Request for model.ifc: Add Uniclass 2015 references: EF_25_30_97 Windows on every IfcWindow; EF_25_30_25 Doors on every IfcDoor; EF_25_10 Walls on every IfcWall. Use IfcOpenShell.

First a look at what the model holds.

```python
import ifcopenshell

model = ifcopenshell.open("model.ifc")
print(model.schema)
print("classifications:", [c.Name for c in model.by_type("IfcClassification")])
for ifc_class in ("IfcDoor", "IfcRoof", "IfcStair", "IfcWall", "IfcWindow"):
    print(ifc_class, len(model.by_type(ifc_class)))
```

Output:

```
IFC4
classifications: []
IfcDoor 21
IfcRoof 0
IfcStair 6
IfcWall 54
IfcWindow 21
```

```python
import ifcopenshell
import ifcopenshell.api.classification

model = ifcopenshell.open("model.ifc")

system = ifcopenshell.api.classification.add_classification(model, classification="Uniclass 2015")

codes = {
    "IfcWindow": ("EF_25_30_97", "Windows"),
    "IfcDoor": ("EF_25_30_25", "Doors"),
    "IfcWall": ("EF_25_10", "Walls"),
}
for ifc_class, (code, name) in codes.items():
    products = model.by_type(ifc_class)
    ifcopenshell.api.classification.add_reference(
        model, products=products, classification=system, identification=code, name=name
    )
    print(code, len(products))

model.write("model-out.ifc")
```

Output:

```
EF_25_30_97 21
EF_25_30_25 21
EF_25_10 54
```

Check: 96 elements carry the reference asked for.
